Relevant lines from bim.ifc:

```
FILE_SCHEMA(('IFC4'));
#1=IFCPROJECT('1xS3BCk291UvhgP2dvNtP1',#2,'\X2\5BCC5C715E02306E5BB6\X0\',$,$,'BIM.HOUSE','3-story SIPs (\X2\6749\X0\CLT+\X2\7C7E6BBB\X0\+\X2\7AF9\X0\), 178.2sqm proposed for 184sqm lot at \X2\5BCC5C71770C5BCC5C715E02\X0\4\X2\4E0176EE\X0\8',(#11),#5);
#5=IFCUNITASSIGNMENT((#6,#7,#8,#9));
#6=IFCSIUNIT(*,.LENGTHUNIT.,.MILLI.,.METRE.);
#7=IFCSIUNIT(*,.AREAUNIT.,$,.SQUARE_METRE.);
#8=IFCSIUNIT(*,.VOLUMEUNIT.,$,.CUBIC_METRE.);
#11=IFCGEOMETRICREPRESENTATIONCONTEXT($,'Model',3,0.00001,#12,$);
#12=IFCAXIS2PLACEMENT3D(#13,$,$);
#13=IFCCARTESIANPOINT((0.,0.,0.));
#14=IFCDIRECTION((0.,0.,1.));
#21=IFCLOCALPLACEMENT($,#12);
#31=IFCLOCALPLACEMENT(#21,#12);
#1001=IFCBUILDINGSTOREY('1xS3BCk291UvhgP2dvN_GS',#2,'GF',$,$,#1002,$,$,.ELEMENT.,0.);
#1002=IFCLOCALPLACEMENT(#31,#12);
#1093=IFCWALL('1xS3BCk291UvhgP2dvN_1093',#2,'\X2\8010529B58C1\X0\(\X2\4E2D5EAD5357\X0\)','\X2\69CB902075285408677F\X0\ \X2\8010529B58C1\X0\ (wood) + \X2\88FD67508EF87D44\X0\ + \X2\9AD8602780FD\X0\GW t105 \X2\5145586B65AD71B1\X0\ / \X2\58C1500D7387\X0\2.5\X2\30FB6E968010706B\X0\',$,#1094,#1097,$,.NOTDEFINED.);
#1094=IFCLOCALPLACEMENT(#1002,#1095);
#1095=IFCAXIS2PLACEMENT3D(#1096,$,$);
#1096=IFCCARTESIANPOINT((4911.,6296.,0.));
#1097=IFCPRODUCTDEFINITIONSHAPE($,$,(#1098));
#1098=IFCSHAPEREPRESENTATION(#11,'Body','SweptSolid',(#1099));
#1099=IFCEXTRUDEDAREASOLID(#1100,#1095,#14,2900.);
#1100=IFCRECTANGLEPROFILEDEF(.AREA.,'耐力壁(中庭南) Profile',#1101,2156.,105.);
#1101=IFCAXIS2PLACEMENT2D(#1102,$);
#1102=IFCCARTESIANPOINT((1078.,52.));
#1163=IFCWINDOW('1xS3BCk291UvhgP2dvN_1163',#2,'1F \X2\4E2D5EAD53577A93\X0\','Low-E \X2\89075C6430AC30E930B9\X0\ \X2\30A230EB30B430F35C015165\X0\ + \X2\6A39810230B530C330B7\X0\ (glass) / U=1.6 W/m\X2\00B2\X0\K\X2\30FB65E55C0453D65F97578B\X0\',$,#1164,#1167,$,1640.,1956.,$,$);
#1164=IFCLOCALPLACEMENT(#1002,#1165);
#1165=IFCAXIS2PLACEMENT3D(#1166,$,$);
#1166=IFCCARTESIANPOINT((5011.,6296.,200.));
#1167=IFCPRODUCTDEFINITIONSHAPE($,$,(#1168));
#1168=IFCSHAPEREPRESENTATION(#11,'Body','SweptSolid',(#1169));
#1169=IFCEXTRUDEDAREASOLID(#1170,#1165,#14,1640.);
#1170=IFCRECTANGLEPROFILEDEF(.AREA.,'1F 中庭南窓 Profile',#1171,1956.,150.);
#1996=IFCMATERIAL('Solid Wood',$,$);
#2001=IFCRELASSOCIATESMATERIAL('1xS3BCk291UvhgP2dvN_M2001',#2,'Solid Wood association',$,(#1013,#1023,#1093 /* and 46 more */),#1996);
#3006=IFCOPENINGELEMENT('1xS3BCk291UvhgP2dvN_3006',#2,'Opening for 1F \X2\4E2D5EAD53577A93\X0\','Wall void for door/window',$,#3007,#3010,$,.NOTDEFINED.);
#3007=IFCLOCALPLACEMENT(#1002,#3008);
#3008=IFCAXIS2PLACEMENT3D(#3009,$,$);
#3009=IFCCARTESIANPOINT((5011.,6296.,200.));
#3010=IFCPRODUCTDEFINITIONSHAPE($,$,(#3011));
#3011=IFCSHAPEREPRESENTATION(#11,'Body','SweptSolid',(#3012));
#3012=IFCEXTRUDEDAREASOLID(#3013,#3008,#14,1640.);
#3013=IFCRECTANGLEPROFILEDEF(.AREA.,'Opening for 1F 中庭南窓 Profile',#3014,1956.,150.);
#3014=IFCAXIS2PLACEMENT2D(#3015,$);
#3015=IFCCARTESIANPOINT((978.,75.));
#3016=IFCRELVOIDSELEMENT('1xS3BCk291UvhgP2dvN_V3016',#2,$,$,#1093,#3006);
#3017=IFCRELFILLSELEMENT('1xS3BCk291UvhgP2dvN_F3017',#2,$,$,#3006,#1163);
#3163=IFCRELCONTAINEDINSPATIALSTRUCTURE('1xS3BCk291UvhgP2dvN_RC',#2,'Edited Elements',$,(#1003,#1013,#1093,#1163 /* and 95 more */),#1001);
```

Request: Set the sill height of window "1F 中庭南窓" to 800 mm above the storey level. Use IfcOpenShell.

```python
import numpy as np
import ifcopenshell
import ifcopenshell.api.geometry
import ifcopenshell.geom
import ifcopenshell.util.element
import ifcopenshell.util.placement
import ifcopenshell.util.shape
import ifcopenshell.util.unit

model = ifcopenshell.open("bim.ifc")
unit_scale = ifcopenshell.util.unit.calculate_unit_scale(model)

window = model.by_guid("1xS3BCk291UvhgP2dvN_1163")
opening = window.FillsVoids[0].RelatingOpeningElement
storey = ifcopenshell.util.element.get_container(window, ifc_class="IfcBuildingStorey")
level = ifcopenshell.util.placement.get_local_placement(storey.ObjectPlacement)[2, 3]

# The opening's origin need not be at the sill, so measure its lowest point.
shape = ifcopenshell.geom.create_shape(ifcopenshell.geom.settings(), opening)
bottom = ifcopenshell.util.shape.get_shape_bottom_elevation(shape, shape.geometry) / unit_scale
dz = level + 0.8 / unit_scale - bottom

shift = np.array([0.0, 0.0, dz])
# The window is not placed relative to its opening, so move both.
for product in (opening, window):
    matrix = ifcopenshell.util.placement.get_local_placement(product.ObjectPlacement)
    matrix[:3, 3] += shift
    ifcopenshell.api.geometry.edit_object_placement(model, product=product, matrix=matrix, is_si=False)

print(f"moved by {dz * unit_scale:+.3f} m")

model.write("bim-out.ifc")
```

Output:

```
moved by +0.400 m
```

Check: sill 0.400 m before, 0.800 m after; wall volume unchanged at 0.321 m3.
